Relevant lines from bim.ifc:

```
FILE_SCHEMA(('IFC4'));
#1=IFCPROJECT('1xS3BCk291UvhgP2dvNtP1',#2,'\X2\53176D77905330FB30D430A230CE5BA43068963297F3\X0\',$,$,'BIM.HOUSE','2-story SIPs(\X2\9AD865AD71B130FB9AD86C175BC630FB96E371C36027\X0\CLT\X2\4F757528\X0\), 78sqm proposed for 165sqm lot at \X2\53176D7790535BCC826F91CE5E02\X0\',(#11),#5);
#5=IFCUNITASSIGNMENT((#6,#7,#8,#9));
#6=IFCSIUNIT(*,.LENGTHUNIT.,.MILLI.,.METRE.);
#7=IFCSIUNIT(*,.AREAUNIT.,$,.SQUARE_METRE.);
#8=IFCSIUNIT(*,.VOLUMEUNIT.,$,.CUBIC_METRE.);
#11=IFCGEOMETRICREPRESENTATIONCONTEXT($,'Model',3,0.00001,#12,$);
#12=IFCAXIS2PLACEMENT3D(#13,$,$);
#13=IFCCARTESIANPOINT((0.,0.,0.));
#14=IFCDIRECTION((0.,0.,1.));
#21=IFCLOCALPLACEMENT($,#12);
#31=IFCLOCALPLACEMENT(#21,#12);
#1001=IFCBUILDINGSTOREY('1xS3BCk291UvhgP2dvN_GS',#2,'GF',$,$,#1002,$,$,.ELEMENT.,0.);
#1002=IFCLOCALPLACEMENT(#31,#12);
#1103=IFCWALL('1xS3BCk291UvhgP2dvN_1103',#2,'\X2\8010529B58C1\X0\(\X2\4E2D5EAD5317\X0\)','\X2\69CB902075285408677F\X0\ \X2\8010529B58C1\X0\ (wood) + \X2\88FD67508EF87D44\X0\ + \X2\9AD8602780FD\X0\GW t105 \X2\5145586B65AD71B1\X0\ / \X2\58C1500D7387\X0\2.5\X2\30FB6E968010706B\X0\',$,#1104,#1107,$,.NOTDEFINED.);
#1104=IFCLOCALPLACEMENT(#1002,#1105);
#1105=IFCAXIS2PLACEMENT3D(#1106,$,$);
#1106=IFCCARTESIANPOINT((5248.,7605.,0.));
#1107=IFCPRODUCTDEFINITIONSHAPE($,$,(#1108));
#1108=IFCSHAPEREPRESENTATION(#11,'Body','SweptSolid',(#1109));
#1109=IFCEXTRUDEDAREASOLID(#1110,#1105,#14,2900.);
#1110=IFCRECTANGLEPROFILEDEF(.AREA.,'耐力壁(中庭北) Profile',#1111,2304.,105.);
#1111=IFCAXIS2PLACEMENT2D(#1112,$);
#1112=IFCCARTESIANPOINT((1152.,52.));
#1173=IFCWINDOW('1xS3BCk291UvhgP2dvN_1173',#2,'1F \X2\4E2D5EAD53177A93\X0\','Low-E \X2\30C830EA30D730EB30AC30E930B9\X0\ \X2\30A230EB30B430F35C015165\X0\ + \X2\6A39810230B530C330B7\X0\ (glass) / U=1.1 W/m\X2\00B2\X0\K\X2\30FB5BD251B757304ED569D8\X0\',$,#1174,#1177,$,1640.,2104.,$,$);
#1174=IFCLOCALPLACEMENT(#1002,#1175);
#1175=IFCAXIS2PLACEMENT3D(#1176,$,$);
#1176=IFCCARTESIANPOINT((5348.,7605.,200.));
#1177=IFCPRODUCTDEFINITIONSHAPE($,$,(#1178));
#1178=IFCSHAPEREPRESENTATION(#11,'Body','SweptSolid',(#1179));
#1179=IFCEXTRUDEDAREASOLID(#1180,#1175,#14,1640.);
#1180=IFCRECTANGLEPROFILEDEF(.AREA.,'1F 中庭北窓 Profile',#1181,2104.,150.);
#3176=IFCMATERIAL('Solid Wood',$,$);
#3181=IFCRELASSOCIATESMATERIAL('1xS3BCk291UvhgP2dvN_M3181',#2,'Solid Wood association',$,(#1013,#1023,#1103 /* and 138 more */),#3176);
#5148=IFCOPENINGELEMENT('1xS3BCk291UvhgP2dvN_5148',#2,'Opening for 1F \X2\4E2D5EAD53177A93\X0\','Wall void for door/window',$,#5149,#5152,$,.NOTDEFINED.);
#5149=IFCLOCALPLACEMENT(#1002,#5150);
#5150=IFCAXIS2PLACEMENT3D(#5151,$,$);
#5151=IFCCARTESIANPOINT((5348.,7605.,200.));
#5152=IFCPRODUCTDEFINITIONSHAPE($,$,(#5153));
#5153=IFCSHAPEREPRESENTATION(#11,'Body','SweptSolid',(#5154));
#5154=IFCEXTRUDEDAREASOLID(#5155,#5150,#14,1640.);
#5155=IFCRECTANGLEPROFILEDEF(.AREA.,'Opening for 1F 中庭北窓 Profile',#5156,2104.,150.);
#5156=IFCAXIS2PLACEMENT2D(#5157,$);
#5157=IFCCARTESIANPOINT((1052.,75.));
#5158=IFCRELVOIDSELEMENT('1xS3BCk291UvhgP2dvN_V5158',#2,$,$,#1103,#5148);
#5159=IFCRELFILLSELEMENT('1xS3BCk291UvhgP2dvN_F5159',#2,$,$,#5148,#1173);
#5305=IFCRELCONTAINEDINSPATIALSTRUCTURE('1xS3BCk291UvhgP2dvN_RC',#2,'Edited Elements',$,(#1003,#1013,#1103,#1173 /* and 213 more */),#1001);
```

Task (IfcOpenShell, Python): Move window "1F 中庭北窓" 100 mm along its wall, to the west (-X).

```python
import ifcopenshell
import ifcopenshell.api.geometry
import ifcopenshell.util.placement
import ifcopenshell.util.unit

model = ifcopenshell.open("bim.ifc")
unit_scale = ifcopenshell.util.unit.calculate_unit_scale(model)

window = model.by_guid("1xS3BCk291UvhgP2dvN_1173")
opening = window.FillsVoids[0].RelatingOpeningElement
wall = opening.VoidsElements[0].RelatingBuildingElement

wall_matrix = ifcopenshell.util.placement.get_local_placement(wall.ObjectPlacement)
shift = wall_matrix[:3, 0] * -0.1 / unit_scale
before = ifcopenshell.util.placement.get_local_placement(window.ObjectPlacement)[:3, 3].copy()

# The window is not placed relative to its opening, so move both.
for product in (opening, window):
    matrix = ifcopenshell.util.placement.get_local_placement(product.ObjectPlacement)
    matrix[:3, 3] += shift
    ifcopenshell.api.geometry.edit_object_placement(model, product=product, matrix=matrix, is_si=False)

after = ifcopenshell.util.placement.get_local_placement(window.ObjectPlacement)[:3, 3]
print("window moved by", (after - before).round(3) + 0.0)

model.write("bim_edited.ifc")
```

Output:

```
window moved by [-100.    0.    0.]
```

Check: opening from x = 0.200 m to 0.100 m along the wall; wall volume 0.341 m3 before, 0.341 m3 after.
